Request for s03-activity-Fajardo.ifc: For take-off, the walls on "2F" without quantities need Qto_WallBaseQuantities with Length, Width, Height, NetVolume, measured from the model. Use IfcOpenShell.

First a look at what the model holds.

```python
import ifcopenshell
import ifcopenshell.util.element
import ifcopenshell.util.unit

model = ifcopenshell.open("s03-activity-Fajardo.ifc")
print(model.schema)
for unit_type in ("LENGTHUNIT", "AREAUNIT", "VOLUMEUNIT"):
    print(unit_type, ifcopenshell.util.unit.calculate_unit_scale(model, unit_type))
storey = next(s for s in model.by_type("IfcBuildingStorey") if s.Name == "2F")
walls = [e for e in ifcopenshell.util.element.get_decomposition(storey) if e.is_a("IfcWall")]
for e in sorted(walls, key=lambda e: e.id()):
    print(e.id(), e.is_a(), e.Name, list(ifcopenshell.util.element.get_psets(e, qtos_only=True)), sep=" | ")
```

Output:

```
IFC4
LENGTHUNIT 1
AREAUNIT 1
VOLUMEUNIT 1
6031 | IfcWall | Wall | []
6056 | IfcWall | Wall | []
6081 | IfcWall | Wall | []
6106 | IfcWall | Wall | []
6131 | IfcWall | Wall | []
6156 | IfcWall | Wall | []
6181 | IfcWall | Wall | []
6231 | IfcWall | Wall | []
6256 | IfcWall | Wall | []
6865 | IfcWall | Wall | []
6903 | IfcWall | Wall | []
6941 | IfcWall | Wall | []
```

```python
import ifcopenshell
import ifcopenshell.api.pset
import ifcopenshell.geom
import ifcopenshell.util.element
import ifcopenshell.util.shape
import ifcopenshell.util.unit

model = ifcopenshell.open("s03-activity-Fajardo.ifc")
unit_scale = ifcopenshell.util.unit.calculate_unit_scale(model)
volume_scale = ifcopenshell.util.unit.calculate_unit_scale(model, "VOLUMEUNIT")
settings = ifcopenshell.geom.settings()

storey = next(s for s in model.by_type("IfcBuildingStorey") if s.Name == "2F")
walls = [e for e in ifcopenshell.util.element.get_decomposition(storey) if e.is_a("IfcWall")]

for e in sorted(walls, key=lambda e: e.id()):
    if ifcopenshell.util.element.get_psets(e, qtos_only=True, should_inherit=False):
        continue
    # Geometry comes back in metres, in the element's own axes.
    shape = ifcopenshell.geom.create_shape(settings, e)
    values = {
        "Length": ifcopenshell.util.shape.get_x(shape.geometry) / unit_scale,
        "Width": ifcopenshell.util.shape.get_y(shape.geometry) / unit_scale,
        "Height": ifcopenshell.util.shape.get_z(shape.geometry) / unit_scale,
        "NetVolume": ifcopenshell.util.shape.get_volume(shape.geometry) / volume_scale,
    }
    qto = ifcopenshell.api.pset.add_qto(model, product=e, name="Qto_WallBaseQuantities")
    ifcopenshell.api.pset.edit_qto(model, qto=qto, properties=values)
    print(e.id(), {k: round(v, 3) for k, v in values.items()})

model.write("s03-activity-Fajardo_rev.ifc")
```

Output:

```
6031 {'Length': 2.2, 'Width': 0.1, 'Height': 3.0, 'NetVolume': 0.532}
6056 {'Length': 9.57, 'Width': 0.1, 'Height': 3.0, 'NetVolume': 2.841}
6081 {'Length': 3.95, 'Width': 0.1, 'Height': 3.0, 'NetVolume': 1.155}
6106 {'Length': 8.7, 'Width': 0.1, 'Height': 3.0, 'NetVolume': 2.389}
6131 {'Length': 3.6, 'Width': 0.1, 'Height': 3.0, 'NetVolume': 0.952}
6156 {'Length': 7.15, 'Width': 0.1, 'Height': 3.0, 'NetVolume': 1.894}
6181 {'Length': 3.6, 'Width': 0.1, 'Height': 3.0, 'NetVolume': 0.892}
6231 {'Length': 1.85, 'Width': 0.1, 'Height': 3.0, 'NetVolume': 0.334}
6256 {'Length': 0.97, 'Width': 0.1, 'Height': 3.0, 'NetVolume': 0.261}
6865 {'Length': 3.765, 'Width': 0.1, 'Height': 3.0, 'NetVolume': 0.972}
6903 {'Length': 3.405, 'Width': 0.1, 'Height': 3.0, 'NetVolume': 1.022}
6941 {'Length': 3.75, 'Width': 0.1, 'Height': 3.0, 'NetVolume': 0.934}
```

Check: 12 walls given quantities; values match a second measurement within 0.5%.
